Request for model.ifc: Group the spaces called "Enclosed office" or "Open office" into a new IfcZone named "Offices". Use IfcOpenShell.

First a look at what the model holds.

```python
import ifcopenshell

model = ifcopenshell.open("model.ifc")
print(model.schema)
seen = {}
for space in model.by_type("IfcSpace"):
    seen[space.LongName] = seen.get(space.LongName, 0) + 1
for name, count in sorted(seen.items(), key=str):
    print(count, "x", name)
print("zones:", [z.Name for z in model.by_type("IfcZone")][:20])
```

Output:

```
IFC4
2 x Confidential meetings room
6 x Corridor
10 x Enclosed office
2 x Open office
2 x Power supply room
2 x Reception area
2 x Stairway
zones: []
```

```python
import ifcopenshell
import ifcopenshell.api.group
import ifcopenshell.api.root

model = ifcopenshell.open("model.ifc")

names = {"Enclosed office", "Open office"}
spaces = [s for s in model.by_type("IfcSpace") if s.LongName in names]

zone = ifcopenshell.api.root.create_entity(model, ifc_class="IfcZone", name="Offices")
ifcopenshell.api.group.assign_group(model, products=spaces, group=zone)
print(len(spaces), "spaces in", zone.Name)

model.write("model_updated.ifc")
```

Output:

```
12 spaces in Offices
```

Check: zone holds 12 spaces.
